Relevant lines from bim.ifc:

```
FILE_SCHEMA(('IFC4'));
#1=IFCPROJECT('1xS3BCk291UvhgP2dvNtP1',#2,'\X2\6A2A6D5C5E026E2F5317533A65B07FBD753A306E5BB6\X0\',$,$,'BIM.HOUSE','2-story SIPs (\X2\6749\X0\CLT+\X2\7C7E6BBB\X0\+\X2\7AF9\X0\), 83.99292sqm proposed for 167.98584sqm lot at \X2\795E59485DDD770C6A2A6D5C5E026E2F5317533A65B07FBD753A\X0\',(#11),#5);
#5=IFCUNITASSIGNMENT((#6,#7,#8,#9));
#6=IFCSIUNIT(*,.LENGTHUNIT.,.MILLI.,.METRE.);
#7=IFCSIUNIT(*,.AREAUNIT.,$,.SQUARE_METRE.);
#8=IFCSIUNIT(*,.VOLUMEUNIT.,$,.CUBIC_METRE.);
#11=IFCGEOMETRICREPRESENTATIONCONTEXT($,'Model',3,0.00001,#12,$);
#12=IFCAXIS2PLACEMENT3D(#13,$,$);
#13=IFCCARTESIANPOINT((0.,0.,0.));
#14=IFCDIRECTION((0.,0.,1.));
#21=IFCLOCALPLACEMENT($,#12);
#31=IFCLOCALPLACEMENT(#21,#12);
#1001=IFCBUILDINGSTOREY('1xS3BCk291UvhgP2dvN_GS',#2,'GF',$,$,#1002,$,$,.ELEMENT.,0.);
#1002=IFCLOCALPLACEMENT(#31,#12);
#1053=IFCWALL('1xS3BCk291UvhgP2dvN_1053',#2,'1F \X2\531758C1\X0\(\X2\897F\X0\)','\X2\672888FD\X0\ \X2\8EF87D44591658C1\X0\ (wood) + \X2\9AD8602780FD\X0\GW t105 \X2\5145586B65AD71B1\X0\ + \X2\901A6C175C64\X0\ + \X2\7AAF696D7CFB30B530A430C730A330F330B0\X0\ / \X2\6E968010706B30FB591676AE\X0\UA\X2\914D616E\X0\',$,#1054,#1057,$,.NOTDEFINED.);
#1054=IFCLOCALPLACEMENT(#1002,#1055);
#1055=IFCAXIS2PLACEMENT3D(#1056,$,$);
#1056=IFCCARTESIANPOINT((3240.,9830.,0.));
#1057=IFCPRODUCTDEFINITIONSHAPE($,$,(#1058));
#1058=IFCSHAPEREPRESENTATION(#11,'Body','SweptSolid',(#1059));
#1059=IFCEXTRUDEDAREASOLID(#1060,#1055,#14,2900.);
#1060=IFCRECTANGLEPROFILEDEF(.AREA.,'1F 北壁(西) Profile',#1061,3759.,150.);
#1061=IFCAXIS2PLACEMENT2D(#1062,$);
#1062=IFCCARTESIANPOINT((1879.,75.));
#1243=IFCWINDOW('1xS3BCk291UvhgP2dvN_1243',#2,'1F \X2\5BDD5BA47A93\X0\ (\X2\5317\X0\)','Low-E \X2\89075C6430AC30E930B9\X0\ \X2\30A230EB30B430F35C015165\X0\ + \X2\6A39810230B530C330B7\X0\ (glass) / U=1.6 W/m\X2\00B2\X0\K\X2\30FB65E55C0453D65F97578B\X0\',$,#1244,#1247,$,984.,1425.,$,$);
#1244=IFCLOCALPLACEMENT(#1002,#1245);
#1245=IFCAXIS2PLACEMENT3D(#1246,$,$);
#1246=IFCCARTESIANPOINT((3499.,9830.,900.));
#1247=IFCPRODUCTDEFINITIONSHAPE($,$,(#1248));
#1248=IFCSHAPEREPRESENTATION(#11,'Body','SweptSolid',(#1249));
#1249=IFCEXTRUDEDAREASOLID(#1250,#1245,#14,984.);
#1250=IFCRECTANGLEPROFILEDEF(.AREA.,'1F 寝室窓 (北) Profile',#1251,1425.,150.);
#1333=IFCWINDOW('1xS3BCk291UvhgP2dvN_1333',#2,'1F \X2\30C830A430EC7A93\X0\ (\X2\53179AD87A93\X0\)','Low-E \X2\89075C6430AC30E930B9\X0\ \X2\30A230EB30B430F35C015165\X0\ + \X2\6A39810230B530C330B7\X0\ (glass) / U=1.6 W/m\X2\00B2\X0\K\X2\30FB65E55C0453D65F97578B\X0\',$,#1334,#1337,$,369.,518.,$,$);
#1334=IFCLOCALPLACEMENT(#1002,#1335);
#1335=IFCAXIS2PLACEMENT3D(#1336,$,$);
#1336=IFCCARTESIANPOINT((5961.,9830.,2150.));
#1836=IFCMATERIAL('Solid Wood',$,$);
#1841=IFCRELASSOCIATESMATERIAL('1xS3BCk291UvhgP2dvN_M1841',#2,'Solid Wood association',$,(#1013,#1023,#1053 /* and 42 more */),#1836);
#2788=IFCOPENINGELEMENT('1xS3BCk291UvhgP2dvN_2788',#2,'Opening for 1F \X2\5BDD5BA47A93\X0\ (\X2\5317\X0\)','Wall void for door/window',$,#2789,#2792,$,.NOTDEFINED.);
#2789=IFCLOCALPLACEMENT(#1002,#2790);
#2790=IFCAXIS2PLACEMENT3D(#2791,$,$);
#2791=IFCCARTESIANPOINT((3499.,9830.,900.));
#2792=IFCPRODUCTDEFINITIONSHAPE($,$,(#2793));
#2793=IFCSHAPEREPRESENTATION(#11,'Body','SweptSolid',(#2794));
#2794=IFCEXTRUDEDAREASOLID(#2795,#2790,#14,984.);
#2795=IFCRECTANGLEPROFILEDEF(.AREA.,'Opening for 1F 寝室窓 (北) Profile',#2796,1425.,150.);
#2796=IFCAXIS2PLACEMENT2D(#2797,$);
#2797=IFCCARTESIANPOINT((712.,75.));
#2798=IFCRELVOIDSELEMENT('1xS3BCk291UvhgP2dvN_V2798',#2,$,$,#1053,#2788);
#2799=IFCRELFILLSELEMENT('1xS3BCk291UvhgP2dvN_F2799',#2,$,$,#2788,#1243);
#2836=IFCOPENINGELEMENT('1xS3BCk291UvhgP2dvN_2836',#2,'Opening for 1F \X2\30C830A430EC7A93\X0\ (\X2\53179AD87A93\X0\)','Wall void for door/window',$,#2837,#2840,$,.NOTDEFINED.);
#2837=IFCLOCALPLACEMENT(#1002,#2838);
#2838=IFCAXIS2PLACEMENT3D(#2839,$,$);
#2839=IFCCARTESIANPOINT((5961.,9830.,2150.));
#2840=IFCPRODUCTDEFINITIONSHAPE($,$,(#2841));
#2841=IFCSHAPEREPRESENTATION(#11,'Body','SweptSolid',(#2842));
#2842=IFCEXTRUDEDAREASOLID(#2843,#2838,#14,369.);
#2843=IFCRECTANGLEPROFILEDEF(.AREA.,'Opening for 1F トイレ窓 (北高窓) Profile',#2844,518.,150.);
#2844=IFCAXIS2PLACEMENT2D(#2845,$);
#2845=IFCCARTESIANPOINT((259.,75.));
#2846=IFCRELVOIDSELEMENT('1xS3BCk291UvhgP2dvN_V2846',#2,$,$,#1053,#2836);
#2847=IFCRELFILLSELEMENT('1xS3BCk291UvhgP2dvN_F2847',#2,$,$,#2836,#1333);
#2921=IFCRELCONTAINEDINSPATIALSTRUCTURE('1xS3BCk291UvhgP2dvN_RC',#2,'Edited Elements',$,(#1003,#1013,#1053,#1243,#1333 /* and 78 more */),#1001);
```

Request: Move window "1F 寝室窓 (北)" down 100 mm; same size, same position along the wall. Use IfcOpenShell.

```python
import numpy as np
import ifcopenshell
import ifcopenshell.api.geometry
import ifcopenshell.util.placement
import ifcopenshell.util.unit

model = ifcopenshell.open("bim.ifc")
unit_scale = ifcopenshell.util.unit.calculate_unit_scale(model)

window = model.by_id(1243)
opening = window.FillsVoids[0].RelatingOpeningElement
dz = -0.1 / unit_scale

shift = np.array([0.0, 0.0, dz])
# The window is not placed relative to its opening, so move both.
for product in (opening, window):
    matrix = ifcopenshell.util.placement.get_local_placement(product.ObjectPlacement)
    matrix[:3, 3] += shift
    ifcopenshell.api.geometry.edit_object_placement(model, product=product, matrix=matrix, is_si=False)

print(f"moved by {dz * unit_scale:+.3f} m")

model.write("bim_edited.ifc")
```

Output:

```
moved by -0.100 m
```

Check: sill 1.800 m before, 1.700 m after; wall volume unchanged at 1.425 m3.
